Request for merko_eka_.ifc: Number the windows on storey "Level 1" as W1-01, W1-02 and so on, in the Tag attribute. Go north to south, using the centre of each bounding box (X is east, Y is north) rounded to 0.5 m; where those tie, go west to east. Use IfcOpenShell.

First a look at what the model holds.

```python
import ifcopenshell
import ifcopenshell.util.element
import ifcopenshell.util.placement

model = ifcopenshell.open("merko_eka_.ifc")
print(model.schema)
storey = next(s for s in model.by_type("IfcBuildingStorey") if s.Name == "Level 1")
windows = [e for e in ifcopenshell.util.element.get_decomposition(storey) if e.is_a("IfcWindow")]
for e in sorted(windows, key=lambda e: e.id()):
    origin = ifcopenshell.util.placement.get_local_placement(e.ObjectPlacement)[:3, 3]
    print(e.id(), e.Tag, e.Name, origin.round(2) + 0.0, sep=" | ")
```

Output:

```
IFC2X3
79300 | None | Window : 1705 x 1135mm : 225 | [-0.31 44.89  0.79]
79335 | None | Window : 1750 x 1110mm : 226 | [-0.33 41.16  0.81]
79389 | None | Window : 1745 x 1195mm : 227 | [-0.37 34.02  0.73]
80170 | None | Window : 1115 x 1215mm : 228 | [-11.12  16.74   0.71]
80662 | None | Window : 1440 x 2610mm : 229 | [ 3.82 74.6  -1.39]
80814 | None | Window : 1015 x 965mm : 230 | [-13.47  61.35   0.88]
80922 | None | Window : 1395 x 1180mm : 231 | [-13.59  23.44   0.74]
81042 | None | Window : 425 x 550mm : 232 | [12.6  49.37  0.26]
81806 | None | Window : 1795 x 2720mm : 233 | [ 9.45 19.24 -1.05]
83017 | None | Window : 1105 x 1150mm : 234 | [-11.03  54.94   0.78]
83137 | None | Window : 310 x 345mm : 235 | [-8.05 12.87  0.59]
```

```python
import ifcopenshell
import ifcopenshell.geom
import ifcopenshell.util.element
import ifcopenshell.util.shape

model = ifcopenshell.open("merko_eka_.ifc")
settings = ifcopenshell.geom.settings()
settings.set("use-world-coords", True)


def centre(element):
    shape = ifcopenshell.geom.create_shape(settings, element)
    return ifcopenshell.util.shape.get_bbox_centroid(shape.geometry)


storey = next(s for s in model.by_type("IfcBuildingStorey") if s.Name == "Level 1")
windows = [e for e in ifcopenshell.util.element.get_decomposition(storey) if e.is_a("IfcWindow")]

# Insertion points can sit at a corner or the storey origin, so sort by the geometry (in metres).
centres = {e: centre(e) for e in windows}
windows.sort(key=lambda e: (-round(centres[e][1] / 0.5), centres[e][0]))

for i, e in enumerate(windows, start=1):
    number = f"W1-{i:02d}"
    e.Tag = number
    print(e.id(), number)

model.write("merko_eka__edited.ifc")
```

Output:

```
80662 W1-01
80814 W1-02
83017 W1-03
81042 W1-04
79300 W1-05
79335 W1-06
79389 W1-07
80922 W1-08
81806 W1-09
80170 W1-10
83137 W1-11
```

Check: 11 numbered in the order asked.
